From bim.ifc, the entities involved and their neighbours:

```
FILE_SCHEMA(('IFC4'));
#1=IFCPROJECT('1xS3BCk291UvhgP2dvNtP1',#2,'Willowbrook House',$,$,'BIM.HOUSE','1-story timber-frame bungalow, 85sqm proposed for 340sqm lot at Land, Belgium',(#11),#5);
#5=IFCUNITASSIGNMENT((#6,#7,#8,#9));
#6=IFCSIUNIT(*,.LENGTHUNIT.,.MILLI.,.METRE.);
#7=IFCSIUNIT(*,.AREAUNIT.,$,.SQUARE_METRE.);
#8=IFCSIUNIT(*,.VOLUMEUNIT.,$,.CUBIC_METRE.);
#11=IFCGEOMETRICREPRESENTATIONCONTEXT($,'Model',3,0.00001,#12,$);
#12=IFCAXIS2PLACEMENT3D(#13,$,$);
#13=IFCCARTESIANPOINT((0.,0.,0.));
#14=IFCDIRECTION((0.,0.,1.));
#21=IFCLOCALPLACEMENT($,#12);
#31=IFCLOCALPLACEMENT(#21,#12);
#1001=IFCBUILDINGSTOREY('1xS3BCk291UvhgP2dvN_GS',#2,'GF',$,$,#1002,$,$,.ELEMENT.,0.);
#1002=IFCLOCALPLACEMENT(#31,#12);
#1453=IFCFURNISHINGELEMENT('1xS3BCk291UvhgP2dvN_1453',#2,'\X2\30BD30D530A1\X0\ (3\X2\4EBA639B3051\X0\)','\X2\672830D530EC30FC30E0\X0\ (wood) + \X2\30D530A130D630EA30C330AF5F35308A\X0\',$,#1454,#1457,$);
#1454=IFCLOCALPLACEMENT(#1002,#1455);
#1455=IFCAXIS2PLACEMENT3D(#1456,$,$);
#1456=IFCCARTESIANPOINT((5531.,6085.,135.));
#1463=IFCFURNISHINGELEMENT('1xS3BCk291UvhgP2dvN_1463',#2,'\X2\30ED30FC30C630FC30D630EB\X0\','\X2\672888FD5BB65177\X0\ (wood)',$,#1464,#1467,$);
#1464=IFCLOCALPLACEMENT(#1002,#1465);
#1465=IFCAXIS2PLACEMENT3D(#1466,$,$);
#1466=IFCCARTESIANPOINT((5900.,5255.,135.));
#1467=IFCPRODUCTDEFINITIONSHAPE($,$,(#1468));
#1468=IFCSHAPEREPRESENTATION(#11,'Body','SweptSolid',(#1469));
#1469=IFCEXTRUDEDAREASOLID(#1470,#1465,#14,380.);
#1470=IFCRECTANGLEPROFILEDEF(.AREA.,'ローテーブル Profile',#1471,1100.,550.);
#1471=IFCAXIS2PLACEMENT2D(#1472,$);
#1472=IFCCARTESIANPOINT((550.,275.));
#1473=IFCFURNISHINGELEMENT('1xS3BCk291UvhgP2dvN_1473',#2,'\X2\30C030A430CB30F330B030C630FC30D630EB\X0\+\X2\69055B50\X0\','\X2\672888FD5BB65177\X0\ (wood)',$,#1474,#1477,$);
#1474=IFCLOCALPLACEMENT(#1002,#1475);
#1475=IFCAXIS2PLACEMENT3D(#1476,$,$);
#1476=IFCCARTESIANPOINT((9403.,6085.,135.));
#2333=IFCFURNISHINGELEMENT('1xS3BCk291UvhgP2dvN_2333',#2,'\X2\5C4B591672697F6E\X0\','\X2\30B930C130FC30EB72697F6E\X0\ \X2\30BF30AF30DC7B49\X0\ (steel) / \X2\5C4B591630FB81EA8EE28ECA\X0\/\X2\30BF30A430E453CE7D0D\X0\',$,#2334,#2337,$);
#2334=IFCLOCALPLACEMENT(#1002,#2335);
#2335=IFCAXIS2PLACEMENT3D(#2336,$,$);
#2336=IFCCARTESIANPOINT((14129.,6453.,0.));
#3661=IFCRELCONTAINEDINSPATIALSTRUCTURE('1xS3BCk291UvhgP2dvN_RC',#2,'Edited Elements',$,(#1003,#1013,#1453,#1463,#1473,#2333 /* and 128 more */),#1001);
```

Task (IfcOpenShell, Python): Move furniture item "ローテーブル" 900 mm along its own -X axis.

```python
import ifcopenshell
import ifcopenshell.api.geometry
import ifcopenshell.util.placement

model = ifcopenshell.open("bim.ifc")

item = model.by_id(1463)
matrix = ifcopenshell.util.placement.get_local_placement(item.ObjectPlacement)
matrix[:3, 3] -= matrix[:3, 0] * 900.0
ifcopenshell.api.geometry.edit_object_placement(model, product=item, matrix=matrix, is_si=False)

print(ifcopenshell.util.placement.get_local_placement(item.ObjectPlacement).round(3) + 0.0)

model.write("bim_rev.ifc")
```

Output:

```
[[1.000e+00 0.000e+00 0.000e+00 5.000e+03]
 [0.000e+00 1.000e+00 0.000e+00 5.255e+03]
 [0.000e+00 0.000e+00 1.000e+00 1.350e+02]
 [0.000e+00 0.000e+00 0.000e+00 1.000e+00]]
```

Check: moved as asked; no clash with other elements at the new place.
